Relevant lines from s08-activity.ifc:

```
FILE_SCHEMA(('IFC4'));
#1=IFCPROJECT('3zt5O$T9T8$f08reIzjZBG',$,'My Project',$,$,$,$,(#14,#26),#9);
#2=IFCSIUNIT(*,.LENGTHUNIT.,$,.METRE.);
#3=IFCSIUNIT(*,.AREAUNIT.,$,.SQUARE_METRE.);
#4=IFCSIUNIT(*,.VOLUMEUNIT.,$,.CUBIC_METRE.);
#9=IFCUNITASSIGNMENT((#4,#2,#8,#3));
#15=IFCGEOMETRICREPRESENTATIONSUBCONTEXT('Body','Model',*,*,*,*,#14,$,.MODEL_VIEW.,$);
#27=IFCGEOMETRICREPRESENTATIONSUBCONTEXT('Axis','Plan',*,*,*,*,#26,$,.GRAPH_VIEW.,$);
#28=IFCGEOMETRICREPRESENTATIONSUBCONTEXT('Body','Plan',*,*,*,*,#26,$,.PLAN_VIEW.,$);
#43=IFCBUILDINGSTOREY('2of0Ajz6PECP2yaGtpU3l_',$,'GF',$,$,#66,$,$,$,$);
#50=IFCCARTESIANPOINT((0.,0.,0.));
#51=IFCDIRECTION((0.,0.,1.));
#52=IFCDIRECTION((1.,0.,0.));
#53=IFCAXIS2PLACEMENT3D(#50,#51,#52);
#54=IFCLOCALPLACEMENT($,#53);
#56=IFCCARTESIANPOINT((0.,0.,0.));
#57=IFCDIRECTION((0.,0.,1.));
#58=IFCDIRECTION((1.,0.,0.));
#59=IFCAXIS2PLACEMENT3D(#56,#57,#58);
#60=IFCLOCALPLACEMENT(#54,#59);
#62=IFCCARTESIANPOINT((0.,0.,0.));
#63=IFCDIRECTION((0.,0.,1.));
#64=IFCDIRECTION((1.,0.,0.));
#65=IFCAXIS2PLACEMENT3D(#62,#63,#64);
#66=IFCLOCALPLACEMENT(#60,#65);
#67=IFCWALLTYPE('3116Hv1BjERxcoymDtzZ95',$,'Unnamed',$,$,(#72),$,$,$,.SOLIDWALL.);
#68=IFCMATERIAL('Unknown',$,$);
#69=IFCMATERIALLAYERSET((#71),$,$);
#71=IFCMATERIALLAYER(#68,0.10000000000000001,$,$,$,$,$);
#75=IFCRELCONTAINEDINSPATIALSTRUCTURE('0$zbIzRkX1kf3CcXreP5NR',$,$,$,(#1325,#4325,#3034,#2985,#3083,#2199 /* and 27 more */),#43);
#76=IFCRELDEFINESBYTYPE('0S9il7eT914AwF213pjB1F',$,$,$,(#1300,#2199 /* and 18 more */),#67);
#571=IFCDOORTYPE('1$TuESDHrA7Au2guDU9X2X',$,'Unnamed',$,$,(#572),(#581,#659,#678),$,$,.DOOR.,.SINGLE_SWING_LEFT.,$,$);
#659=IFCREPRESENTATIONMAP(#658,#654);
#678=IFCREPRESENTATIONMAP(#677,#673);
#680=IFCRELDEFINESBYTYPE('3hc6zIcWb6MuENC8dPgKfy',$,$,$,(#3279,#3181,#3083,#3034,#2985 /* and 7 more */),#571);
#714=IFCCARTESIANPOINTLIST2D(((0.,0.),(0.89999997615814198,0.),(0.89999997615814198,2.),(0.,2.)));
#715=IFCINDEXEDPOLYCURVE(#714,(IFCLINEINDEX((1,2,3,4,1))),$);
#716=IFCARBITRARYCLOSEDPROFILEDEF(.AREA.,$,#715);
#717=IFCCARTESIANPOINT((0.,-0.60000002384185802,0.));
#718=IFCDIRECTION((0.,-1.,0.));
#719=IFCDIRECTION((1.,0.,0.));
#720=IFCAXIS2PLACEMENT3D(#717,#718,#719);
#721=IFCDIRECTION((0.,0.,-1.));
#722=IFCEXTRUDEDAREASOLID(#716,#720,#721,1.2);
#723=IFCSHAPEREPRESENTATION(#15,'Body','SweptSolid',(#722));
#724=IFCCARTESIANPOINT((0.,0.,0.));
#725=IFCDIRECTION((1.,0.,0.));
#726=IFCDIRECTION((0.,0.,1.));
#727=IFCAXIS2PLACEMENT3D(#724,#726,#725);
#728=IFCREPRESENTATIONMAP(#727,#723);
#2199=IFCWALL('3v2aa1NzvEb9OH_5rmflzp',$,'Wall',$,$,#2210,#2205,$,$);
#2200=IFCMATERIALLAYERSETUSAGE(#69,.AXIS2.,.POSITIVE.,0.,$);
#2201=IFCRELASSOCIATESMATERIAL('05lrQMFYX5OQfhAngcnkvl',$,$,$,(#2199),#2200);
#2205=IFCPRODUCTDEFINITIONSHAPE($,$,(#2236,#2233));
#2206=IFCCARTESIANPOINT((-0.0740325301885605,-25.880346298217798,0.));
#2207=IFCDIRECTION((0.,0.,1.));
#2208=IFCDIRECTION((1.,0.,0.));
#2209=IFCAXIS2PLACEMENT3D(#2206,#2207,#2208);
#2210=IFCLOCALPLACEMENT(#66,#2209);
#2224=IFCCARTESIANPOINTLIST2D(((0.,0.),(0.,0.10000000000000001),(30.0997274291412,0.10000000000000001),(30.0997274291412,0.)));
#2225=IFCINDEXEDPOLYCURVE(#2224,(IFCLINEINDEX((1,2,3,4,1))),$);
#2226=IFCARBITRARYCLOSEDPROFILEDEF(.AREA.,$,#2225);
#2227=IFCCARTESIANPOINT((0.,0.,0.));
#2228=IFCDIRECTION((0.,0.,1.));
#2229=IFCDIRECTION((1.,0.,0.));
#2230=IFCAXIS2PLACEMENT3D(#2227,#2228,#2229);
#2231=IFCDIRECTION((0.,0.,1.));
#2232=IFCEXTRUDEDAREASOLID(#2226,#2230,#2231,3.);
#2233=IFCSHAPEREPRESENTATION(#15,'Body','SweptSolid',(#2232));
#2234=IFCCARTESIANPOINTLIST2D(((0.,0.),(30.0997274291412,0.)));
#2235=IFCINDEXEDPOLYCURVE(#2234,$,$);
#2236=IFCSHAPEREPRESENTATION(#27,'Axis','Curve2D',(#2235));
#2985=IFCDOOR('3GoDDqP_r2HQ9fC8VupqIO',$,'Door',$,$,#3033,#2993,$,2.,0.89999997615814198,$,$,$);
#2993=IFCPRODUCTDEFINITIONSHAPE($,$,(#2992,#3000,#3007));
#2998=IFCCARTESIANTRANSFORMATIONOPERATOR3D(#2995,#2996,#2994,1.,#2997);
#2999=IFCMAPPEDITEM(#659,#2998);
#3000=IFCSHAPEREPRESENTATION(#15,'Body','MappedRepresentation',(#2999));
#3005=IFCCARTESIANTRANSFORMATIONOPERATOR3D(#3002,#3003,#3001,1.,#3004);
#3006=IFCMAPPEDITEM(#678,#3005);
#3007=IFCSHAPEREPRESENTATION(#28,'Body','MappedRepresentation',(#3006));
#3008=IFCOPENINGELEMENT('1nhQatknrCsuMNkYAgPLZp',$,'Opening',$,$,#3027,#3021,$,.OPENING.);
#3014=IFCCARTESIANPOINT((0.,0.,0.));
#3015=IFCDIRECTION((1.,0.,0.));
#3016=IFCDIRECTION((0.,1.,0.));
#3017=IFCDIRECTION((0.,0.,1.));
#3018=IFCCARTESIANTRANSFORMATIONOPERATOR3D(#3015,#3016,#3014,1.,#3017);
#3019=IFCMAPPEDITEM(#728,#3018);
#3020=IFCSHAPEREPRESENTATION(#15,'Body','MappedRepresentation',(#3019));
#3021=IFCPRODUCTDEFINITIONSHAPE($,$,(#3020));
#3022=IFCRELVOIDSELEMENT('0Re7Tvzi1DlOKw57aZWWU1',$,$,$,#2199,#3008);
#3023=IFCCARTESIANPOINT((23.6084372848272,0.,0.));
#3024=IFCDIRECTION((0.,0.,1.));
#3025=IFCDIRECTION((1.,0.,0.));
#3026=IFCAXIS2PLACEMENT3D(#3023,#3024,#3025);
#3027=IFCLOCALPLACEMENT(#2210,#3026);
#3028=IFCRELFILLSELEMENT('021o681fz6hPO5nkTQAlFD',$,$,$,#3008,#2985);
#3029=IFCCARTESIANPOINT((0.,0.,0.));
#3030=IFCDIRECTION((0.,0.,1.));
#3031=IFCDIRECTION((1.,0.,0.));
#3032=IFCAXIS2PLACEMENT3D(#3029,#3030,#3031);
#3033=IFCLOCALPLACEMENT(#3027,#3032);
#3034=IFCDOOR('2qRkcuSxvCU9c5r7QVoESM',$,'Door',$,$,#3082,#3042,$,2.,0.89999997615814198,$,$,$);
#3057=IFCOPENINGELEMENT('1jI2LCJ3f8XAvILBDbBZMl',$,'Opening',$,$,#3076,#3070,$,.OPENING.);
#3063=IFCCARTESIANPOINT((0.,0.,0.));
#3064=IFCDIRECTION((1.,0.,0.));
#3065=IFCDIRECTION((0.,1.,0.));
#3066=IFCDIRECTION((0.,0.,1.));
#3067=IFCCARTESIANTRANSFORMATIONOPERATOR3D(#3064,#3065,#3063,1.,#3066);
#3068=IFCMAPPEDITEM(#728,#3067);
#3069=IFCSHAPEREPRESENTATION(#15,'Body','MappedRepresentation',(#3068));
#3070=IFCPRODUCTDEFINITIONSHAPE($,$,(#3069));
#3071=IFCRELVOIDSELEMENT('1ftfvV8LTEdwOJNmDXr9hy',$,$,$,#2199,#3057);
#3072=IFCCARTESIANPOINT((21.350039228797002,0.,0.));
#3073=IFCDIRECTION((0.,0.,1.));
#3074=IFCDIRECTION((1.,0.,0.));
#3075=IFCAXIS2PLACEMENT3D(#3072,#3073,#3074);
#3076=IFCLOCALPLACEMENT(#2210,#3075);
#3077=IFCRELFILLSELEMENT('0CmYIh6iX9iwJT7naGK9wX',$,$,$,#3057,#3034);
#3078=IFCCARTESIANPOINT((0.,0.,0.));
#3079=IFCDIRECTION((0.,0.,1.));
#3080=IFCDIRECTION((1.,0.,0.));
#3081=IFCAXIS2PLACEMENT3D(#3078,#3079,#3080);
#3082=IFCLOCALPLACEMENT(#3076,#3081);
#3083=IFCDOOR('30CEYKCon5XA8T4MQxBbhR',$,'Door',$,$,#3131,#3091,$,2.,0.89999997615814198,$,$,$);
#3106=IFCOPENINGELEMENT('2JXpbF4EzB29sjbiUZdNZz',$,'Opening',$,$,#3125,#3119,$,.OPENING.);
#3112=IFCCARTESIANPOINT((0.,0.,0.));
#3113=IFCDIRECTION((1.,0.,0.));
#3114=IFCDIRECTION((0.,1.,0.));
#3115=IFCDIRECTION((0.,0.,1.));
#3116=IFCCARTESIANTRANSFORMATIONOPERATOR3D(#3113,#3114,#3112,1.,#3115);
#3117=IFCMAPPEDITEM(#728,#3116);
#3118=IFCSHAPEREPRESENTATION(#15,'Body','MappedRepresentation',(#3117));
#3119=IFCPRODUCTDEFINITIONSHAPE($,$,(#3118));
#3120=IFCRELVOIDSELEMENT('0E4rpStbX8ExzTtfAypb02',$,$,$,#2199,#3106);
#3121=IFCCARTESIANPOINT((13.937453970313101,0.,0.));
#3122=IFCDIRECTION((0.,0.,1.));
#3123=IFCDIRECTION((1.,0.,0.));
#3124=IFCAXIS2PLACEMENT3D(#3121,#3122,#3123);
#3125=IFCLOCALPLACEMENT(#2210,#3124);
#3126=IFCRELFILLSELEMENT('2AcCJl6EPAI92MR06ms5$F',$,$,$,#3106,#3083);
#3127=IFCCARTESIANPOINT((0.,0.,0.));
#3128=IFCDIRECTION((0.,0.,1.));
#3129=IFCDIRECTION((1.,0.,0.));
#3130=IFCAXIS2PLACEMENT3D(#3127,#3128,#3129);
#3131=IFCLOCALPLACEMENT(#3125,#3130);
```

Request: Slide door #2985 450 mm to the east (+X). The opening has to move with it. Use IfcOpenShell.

```python
import ifcopenshell
import ifcopenshell.api.geometry
import ifcopenshell.util.placement

model = ifcopenshell.open("s08-activity.ifc")

door = model.by_guid("3GoDDqP_r2HQ9fC8VupqIO")
opening = door.FillsVoids[0].RelatingOpeningElement
wall = opening.VoidsElements[0].RelatingBuildingElement

wall_matrix = ifcopenshell.util.placement.get_local_placement(wall.ObjectPlacement)
shift = wall_matrix[:3, 0] * 0.45
before = ifcopenshell.util.placement.get_local_placement(door.ObjectPlacement)[:3, 3].copy()

# The door is placed relative to its opening, so it follows when the opening moves.
matrix = ifcopenshell.util.placement.get_local_placement(opening.ObjectPlacement)
matrix[:3, 3] += shift
ifcopenshell.api.geometry.edit_object_placement(
    model, product=opening, matrix=matrix, is_si=False, should_transform_children=True
)

after = ifcopenshell.util.placement.get_local_placement(door.ObjectPlacement)[:3, 3]
print("door moved by", (after - before).round(3) + 0.0)

model.write("s08-activity-out.ifc")
```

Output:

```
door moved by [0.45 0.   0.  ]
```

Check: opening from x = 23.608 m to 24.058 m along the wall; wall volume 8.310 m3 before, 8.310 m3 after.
